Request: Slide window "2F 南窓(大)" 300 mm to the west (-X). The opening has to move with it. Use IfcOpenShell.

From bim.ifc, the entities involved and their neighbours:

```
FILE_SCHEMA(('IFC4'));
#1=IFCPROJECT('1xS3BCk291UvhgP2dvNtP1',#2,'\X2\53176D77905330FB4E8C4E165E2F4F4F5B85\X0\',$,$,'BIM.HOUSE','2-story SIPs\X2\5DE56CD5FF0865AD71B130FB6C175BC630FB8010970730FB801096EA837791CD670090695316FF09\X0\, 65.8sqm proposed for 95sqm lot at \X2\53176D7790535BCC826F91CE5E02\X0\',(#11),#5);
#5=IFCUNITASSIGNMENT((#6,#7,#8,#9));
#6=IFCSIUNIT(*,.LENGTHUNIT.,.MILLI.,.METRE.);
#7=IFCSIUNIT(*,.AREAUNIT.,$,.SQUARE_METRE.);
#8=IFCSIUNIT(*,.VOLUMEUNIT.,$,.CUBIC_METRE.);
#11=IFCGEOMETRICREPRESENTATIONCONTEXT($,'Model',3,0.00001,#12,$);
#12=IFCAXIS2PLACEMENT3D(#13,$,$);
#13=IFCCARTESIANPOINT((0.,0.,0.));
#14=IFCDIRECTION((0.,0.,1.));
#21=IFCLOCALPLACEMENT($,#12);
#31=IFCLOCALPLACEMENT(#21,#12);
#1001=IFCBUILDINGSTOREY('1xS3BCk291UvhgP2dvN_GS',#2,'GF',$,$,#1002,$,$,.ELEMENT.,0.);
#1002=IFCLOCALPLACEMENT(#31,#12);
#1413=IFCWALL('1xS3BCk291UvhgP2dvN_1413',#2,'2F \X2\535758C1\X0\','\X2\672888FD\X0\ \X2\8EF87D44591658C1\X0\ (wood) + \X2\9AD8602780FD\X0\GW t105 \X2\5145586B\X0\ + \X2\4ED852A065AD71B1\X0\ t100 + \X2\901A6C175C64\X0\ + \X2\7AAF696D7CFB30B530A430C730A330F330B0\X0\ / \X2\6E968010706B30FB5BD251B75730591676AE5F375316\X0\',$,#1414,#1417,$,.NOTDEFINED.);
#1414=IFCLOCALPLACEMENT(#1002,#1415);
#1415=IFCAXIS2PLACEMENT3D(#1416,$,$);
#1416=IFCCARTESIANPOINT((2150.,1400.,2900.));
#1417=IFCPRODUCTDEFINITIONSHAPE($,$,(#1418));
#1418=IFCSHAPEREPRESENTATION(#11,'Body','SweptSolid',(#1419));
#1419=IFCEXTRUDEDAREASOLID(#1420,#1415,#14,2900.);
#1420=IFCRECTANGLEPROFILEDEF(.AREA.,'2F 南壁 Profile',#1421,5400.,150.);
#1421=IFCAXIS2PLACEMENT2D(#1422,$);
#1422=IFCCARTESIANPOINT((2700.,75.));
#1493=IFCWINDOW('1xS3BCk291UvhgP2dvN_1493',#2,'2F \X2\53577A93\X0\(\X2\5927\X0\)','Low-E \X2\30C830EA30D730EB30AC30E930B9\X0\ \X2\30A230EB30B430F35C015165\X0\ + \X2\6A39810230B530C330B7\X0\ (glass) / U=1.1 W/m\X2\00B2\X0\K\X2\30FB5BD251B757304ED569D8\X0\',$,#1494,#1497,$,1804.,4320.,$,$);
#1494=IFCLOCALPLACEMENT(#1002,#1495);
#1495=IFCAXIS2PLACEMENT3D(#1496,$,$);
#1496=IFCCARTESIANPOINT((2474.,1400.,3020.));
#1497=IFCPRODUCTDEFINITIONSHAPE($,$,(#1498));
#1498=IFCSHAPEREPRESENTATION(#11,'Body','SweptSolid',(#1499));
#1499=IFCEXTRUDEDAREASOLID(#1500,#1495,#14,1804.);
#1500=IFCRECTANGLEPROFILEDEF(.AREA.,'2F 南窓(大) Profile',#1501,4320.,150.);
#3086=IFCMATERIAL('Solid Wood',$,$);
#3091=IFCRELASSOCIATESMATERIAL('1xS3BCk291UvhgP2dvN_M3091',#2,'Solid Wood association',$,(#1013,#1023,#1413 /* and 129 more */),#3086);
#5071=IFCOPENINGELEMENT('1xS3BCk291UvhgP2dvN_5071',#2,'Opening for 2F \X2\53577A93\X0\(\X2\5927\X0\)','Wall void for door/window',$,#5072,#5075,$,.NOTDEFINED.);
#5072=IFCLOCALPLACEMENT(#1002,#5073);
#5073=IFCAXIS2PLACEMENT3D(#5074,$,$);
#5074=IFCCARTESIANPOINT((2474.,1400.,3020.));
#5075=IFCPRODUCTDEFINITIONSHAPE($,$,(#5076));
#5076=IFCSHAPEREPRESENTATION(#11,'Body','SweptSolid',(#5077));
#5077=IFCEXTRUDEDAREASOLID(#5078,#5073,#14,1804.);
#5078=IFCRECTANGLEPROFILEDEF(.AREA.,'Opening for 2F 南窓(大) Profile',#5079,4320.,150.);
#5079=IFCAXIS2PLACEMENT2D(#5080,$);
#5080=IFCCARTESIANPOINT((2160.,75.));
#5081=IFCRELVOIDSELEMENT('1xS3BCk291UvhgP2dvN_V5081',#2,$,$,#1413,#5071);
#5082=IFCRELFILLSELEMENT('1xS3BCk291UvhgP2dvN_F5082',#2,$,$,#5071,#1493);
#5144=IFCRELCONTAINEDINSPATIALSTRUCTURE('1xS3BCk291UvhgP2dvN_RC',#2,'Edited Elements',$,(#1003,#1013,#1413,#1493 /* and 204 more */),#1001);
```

```python
import ifcopenshell
import ifcopenshell.api.geometry
import ifcopenshell.util.placement

model = ifcopenshell.open("bim.ifc")

window = model.by_guid("1xS3BCk291UvhgP2dvN_1493")
opening = window.FillsVoids[0].RelatingOpeningElement
wall = opening.VoidsElements[0].RelatingBuildingElement

wall_matrix = ifcopenshell.util.placement.get_local_placement(wall.ObjectPlacement)
shift = wall_matrix[:3, 0] * -300.0
before = ifcopenshell.util.placement.get_local_placement(window.ObjectPlacement)[:3, 3].copy()

# The window is not placed relative to its opening, so move both.
for product in (opening, window):
    matrix = ifcopenshell.util.placement.get_local_placement(product.ObjectPlacement)
    matrix[:3, 3] += shift
    ifcopenshell.api.geometry.edit_object_placement(model, product=product, matrix=matrix, is_si=False)

after = ifcopenshell.util.placement.get_local_placement(window.ObjectPlacement)[:3, 3]
print("window moved by", (after - before).round(3) + 0.0)

model.write("bim_edited.ifc")
```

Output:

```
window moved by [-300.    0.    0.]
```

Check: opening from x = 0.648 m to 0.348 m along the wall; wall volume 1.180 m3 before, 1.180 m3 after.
